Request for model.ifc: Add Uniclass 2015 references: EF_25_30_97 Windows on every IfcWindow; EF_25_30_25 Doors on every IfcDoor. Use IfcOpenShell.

First a look at what the model holds.

```python
import ifcopenshell

model = ifcopenshell.open("model.ifc")
print(model.schema)
print("classifications:", [c.Name for c in model.by_type("IfcClassification")])
for ifc_class in ("IfcDoor", "IfcRoof", "IfcStair", "IfcWall", "IfcWindow"):
    print(ifc_class, len(model.by_type(ifc_class)))
```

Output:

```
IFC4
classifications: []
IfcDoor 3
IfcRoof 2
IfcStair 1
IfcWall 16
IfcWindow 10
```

```python
import ifcopenshell
import ifcopenshell.api.classification

model = ifcopenshell.open("model.ifc")

system = ifcopenshell.api.classification.add_classification(model, classification="Uniclass 2015")

codes = {
    "IfcWindow": ("EF_25_30_97", "Windows"),
    "IfcDoor": ("EF_25_30_25", "Doors"),
}
for ifc_class, (code, name) in codes.items():
    products = model.by_type(ifc_class)
    ifcopenshell.api.classification.add_reference(
        model, products=products, classification=system, identification=code, name=name
    )
    print(code, len(products))

model.write("model-out.ifc")
```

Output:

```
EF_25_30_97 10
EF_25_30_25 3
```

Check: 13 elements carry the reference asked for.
